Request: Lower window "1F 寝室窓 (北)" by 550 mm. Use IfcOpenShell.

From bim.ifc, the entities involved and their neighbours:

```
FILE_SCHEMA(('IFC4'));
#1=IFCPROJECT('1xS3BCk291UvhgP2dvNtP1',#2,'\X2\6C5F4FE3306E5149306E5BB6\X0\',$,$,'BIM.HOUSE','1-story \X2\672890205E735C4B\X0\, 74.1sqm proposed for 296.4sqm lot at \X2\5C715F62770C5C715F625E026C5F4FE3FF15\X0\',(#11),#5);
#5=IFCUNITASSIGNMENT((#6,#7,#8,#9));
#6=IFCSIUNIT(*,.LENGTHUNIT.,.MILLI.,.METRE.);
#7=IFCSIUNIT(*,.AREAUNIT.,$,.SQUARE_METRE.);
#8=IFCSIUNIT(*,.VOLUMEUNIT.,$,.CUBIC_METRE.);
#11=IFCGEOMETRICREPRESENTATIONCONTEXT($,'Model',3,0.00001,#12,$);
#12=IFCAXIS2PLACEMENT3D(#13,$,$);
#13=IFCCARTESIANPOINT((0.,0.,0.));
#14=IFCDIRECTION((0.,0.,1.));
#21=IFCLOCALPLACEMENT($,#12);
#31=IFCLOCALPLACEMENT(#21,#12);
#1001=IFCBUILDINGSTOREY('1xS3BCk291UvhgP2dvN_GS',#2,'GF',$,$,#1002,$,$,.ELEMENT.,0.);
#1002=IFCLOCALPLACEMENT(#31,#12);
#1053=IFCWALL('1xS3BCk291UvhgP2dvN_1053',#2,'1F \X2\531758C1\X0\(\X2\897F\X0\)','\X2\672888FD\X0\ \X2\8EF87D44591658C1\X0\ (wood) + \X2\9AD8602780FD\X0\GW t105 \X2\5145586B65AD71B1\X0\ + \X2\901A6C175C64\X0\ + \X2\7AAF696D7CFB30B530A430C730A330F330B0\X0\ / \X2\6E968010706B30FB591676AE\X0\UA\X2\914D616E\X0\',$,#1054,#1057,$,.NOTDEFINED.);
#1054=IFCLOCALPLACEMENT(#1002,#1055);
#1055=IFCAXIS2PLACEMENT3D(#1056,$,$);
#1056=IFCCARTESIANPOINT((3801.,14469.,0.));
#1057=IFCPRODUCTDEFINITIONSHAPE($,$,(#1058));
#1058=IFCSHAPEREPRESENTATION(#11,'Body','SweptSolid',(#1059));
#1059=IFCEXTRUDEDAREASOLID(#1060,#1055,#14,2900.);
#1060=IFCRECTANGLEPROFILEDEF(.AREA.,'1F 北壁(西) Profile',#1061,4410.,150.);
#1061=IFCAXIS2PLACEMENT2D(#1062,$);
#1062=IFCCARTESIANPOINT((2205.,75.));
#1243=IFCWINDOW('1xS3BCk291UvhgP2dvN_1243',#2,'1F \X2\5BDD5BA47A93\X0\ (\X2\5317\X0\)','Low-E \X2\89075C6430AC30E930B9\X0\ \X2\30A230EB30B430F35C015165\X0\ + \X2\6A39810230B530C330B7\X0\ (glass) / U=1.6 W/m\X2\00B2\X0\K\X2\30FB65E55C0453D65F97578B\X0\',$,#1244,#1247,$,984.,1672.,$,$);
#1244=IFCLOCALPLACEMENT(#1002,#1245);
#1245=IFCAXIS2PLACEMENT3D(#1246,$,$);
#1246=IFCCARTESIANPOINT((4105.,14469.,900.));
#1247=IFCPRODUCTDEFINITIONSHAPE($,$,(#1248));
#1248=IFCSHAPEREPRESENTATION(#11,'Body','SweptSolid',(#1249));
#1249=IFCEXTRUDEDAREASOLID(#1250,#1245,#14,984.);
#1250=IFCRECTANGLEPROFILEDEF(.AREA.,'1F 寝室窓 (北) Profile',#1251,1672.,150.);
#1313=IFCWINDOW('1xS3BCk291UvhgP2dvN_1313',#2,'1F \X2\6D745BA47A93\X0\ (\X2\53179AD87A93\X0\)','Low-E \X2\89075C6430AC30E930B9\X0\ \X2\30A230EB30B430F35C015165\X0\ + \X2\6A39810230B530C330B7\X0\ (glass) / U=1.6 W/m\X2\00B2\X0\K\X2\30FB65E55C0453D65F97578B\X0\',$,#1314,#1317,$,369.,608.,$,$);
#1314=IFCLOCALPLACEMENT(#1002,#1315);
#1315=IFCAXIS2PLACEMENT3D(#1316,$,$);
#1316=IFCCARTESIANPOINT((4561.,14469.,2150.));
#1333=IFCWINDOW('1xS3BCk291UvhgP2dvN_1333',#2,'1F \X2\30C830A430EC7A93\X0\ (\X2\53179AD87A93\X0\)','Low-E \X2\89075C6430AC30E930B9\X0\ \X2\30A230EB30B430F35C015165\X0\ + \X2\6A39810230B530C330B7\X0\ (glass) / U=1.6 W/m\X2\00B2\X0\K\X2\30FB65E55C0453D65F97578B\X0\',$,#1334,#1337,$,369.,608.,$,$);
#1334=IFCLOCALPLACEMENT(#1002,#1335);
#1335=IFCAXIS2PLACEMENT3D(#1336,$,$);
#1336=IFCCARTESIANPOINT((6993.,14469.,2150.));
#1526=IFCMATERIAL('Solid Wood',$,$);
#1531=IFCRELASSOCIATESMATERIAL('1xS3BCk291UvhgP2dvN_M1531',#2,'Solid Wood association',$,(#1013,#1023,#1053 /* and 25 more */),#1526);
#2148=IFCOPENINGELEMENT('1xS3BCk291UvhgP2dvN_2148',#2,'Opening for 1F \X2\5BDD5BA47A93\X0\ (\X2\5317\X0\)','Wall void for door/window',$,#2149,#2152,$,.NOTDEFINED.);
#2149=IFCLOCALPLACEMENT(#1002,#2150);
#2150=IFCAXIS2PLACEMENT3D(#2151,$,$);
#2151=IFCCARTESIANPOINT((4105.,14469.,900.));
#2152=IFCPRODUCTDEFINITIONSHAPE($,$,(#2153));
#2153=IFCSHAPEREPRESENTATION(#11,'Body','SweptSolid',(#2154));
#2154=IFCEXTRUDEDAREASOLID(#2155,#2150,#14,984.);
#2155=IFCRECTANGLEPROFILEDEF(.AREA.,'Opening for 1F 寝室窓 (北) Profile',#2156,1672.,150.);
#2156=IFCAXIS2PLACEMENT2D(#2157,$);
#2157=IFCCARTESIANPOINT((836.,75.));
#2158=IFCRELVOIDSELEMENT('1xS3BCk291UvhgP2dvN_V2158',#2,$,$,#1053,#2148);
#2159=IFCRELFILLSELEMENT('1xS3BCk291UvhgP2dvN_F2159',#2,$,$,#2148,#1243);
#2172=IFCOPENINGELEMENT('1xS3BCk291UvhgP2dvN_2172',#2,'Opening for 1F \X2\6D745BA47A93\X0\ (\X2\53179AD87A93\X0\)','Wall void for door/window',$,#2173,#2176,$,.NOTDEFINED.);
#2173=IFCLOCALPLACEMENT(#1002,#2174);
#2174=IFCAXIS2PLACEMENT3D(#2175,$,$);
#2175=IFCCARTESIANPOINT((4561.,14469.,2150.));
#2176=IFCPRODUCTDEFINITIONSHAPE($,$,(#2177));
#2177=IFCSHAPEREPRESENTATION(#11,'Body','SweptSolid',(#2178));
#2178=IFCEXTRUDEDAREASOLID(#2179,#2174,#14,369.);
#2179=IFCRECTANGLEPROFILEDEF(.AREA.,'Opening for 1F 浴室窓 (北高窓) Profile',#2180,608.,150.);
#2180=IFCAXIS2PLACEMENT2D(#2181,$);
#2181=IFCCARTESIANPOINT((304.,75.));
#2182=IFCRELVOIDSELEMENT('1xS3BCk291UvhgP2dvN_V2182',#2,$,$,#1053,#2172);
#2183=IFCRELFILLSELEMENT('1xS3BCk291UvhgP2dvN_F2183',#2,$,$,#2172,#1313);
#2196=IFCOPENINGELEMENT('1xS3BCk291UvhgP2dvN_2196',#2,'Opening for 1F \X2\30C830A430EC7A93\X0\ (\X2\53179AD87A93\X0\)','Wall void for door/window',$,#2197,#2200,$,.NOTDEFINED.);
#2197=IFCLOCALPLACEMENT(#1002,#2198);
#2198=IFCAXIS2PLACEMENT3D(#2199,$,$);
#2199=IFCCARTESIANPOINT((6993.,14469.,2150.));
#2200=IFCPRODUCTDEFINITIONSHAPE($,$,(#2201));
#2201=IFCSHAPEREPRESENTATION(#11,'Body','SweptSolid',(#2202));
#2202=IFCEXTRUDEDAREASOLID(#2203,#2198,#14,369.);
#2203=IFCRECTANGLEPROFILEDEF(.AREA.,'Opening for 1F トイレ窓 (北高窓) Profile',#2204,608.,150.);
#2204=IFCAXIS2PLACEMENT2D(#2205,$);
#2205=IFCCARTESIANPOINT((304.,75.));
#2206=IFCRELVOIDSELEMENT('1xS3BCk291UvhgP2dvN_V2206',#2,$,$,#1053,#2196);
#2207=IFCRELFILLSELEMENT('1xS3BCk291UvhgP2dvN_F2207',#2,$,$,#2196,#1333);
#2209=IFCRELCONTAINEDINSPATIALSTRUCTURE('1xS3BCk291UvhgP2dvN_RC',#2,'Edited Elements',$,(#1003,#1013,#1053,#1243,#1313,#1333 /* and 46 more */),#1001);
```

```python
import numpy as np
import ifcopenshell
import ifcopenshell.api.geometry
import ifcopenshell.util.placement
import ifcopenshell.util.unit

model = ifcopenshell.open("bim.ifc")
unit_scale = ifcopenshell.util.unit.calculate_unit_scale(model)

window = model.by_guid("1xS3BCk291UvhgP2dvN_1243")
opening = window.FillsVoids[0].RelatingOpeningElement
dz = -0.55 / unit_scale

shift = np.array([0.0, 0.0, dz])
# The window is not placed relative to its opening, so move both.
for product in (opening, window):
    matrix = ifcopenshell.util.placement.get_local_placement(product.ObjectPlacement)
    matrix[:3, 3] += shift
    ifcopenshell.api.geometry.edit_object_placement(model, product=product, matrix=matrix, is_si=False)

print(f"moved by {dz * unit_scale:+.3f} m")

model.write("bim-out.ifc")
```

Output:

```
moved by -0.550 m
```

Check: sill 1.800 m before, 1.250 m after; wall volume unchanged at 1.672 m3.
